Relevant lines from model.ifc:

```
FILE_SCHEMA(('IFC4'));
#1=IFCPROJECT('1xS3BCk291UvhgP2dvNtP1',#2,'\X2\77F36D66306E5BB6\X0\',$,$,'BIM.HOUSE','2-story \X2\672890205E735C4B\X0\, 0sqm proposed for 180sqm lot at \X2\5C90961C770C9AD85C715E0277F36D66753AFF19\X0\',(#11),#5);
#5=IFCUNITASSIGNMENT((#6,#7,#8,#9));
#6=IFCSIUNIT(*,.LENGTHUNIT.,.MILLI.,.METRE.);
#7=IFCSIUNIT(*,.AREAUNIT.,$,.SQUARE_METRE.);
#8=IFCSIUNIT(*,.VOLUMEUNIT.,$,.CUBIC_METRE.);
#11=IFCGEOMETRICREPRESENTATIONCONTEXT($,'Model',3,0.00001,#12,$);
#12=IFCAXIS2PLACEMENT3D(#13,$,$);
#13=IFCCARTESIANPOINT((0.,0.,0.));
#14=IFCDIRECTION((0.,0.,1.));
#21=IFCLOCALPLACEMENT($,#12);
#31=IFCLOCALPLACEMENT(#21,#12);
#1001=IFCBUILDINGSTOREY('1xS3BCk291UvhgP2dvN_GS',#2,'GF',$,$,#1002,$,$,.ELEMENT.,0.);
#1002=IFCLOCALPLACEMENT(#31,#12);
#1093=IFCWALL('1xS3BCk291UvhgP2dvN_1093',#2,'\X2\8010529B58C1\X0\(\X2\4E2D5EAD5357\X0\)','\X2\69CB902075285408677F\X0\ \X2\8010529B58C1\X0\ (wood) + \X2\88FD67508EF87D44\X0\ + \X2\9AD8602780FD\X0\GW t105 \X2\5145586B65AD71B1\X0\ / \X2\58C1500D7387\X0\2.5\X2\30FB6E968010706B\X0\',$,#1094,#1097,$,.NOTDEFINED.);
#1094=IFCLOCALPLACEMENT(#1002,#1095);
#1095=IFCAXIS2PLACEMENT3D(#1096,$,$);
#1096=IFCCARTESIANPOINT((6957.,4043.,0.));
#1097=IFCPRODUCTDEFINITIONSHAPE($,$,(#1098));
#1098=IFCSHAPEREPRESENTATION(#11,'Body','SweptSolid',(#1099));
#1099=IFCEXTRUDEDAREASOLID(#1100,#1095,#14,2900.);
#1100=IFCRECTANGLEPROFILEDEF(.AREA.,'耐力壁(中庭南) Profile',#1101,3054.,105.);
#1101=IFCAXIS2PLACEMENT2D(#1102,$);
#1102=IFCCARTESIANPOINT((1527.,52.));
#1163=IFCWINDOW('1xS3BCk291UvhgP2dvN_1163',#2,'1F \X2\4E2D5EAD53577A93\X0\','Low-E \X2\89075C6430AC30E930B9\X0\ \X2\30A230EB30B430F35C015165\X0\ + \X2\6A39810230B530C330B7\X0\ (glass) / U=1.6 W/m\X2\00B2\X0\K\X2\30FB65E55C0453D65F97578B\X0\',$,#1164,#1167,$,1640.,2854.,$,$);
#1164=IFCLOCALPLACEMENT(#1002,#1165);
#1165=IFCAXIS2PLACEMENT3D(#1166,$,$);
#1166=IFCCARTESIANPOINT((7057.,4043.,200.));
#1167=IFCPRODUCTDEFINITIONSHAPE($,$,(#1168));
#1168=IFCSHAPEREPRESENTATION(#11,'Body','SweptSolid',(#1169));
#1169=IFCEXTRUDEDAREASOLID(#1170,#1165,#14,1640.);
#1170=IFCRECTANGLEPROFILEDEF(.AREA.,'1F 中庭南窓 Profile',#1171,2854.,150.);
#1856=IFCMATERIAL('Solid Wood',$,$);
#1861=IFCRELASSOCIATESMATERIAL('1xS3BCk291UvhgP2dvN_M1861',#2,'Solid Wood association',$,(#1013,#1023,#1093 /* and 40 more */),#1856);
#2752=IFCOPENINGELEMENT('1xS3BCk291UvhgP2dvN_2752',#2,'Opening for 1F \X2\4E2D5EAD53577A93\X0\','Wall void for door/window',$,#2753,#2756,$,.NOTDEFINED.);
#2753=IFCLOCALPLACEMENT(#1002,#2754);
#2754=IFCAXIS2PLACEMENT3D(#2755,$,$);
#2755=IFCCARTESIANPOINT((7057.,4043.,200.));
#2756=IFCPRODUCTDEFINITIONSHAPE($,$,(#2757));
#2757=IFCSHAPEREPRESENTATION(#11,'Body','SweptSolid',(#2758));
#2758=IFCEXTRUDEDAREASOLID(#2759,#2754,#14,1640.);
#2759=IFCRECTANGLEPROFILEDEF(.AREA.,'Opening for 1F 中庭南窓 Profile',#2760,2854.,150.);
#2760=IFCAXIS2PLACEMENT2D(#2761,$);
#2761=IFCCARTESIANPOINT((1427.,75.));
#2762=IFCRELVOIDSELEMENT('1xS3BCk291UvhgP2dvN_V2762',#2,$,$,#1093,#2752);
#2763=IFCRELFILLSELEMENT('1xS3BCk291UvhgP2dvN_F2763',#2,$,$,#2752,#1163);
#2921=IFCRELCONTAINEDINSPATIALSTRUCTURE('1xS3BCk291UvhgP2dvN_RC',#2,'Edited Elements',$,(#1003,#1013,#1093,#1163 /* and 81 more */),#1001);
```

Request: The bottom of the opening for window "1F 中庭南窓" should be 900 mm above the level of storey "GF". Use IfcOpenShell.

```python
import numpy as np
import ifcopenshell
import ifcopenshell.api.geometry
import ifcopenshell.geom
import ifcopenshell.util.element
import ifcopenshell.util.placement
import ifcopenshell.util.shape
import ifcopenshell.util.unit

model = ifcopenshell.open("model.ifc")
unit_scale = ifcopenshell.util.unit.calculate_unit_scale(model)

window = model.by_guid("1xS3BCk291UvhgP2dvN_1163")
opening = window.FillsVoids[0].RelatingOpeningElement
storey = ifcopenshell.util.element.get_container(window, ifc_class="IfcBuildingStorey")
level = ifcopenshell.util.placement.get_local_placement(storey.ObjectPlacement)[2, 3]

# The opening's origin need not be at the sill, so measure its lowest point.
shape = ifcopenshell.geom.create_shape(ifcopenshell.geom.settings(), opening)
bottom = ifcopenshell.util.shape.get_shape_bottom_elevation(shape, shape.geometry) / unit_scale
dz = level + 0.9 / unit_scale - bottom

shift = np.array([0.0, 0.0, dz])
# The window is not placed relative to its opening, so move both.
for product in (opening, window):
    matrix = ifcopenshell.util.placement.get_local_placement(product.ObjectPlacement)
    matrix[:3, 3] += shift
    ifcopenshell.api.geometry.edit_object_placement(model, product=product, matrix=matrix, is_si=False)

print(f"moved by {dz * unit_scale:+.3f} m")

model.write("model_rev.ifc")
```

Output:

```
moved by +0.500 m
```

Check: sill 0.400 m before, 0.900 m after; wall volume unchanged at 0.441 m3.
